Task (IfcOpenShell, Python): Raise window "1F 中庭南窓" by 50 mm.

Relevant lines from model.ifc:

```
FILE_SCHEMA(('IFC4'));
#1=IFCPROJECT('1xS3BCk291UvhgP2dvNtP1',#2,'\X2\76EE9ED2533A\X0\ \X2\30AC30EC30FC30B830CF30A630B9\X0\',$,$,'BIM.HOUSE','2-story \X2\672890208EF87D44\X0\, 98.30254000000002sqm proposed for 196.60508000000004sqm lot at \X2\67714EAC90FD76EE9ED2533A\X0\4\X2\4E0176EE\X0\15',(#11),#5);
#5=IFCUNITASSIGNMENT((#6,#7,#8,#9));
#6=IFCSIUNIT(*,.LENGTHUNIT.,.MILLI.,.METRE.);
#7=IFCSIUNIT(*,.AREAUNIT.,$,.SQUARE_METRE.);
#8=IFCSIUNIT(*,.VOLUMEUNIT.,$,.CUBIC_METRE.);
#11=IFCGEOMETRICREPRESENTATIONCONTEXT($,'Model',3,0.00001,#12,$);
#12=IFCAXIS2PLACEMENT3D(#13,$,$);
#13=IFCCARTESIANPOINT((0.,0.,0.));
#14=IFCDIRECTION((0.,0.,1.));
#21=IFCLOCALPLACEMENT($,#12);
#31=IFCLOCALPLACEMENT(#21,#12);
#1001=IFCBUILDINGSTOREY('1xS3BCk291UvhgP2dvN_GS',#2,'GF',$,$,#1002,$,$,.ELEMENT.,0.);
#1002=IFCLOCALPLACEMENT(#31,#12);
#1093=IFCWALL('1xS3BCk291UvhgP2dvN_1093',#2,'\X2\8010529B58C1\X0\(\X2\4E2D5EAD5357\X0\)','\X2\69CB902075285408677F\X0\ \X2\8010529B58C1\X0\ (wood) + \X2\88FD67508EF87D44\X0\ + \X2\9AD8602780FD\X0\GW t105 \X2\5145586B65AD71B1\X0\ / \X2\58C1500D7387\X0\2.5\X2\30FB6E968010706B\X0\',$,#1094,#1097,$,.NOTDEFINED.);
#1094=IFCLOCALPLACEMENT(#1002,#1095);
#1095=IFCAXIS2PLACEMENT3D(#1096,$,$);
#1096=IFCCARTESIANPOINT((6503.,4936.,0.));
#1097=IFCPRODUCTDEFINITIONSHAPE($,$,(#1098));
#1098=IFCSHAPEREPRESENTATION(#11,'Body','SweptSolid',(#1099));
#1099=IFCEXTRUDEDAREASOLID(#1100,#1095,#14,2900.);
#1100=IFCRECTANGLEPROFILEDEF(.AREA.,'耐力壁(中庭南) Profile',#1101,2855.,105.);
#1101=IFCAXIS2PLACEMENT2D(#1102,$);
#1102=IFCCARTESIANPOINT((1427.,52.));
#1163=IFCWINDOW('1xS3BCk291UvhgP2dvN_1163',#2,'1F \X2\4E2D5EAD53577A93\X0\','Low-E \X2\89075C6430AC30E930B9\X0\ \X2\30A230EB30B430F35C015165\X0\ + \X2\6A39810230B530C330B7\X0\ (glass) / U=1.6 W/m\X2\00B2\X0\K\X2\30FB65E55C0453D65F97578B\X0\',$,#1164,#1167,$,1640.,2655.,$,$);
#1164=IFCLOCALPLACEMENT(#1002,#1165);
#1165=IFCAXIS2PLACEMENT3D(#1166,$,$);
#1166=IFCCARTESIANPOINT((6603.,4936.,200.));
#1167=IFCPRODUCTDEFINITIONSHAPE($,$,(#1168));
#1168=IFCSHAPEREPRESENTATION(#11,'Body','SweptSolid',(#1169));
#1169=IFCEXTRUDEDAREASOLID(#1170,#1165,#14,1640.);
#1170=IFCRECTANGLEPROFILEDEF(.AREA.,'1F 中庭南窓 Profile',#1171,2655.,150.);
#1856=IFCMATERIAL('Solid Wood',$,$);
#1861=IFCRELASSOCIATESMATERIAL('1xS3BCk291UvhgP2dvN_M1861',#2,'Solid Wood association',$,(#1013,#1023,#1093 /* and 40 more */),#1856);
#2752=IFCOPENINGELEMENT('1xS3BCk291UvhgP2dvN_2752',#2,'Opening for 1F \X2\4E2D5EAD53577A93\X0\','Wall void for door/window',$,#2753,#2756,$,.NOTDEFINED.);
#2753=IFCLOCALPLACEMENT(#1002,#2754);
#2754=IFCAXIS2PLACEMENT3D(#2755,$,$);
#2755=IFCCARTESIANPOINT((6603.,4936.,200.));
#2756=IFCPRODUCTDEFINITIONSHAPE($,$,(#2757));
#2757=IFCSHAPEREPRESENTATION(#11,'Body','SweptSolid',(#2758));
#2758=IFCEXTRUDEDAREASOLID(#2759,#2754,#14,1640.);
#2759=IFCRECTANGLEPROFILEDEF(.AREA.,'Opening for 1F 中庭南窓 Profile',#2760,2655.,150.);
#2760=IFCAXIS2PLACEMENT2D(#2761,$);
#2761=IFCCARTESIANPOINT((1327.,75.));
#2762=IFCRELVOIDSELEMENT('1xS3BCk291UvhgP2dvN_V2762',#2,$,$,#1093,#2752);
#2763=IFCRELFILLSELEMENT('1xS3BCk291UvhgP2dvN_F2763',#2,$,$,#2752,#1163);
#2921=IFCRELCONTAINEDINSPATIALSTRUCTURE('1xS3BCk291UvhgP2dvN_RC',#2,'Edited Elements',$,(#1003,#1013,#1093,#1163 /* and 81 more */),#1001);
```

```python
import numpy as np
import ifcopenshell
import ifcopenshell.api.geometry
import ifcopenshell.util.placement
import ifcopenshell.util.unit

model = ifcopenshell.open("model.ifc")
unit_scale = ifcopenshell.util.unit.calculate_unit_scale(model)

window = model.by_id(1163)
opening = window.FillsVoids[0].RelatingOpeningElement
dz = 50.0

shift = np.array([0.0, 0.0, dz])
# The window is not placed relative to its opening, so move both.
for product in (opening, window):
    matrix = ifcopenshell.util.placement.get_local_placement(product.ObjectPlacement)
    matrix[:3, 3] += shift
    ifcopenshell.api.geometry.edit_object_placement(model, product=product, matrix=matrix, is_si=False)

print(f"moved by {dz * unit_scale:+.3f} m")

model.write("model_rev.ifc")
```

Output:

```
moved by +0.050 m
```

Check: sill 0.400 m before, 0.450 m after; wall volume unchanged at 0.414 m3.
